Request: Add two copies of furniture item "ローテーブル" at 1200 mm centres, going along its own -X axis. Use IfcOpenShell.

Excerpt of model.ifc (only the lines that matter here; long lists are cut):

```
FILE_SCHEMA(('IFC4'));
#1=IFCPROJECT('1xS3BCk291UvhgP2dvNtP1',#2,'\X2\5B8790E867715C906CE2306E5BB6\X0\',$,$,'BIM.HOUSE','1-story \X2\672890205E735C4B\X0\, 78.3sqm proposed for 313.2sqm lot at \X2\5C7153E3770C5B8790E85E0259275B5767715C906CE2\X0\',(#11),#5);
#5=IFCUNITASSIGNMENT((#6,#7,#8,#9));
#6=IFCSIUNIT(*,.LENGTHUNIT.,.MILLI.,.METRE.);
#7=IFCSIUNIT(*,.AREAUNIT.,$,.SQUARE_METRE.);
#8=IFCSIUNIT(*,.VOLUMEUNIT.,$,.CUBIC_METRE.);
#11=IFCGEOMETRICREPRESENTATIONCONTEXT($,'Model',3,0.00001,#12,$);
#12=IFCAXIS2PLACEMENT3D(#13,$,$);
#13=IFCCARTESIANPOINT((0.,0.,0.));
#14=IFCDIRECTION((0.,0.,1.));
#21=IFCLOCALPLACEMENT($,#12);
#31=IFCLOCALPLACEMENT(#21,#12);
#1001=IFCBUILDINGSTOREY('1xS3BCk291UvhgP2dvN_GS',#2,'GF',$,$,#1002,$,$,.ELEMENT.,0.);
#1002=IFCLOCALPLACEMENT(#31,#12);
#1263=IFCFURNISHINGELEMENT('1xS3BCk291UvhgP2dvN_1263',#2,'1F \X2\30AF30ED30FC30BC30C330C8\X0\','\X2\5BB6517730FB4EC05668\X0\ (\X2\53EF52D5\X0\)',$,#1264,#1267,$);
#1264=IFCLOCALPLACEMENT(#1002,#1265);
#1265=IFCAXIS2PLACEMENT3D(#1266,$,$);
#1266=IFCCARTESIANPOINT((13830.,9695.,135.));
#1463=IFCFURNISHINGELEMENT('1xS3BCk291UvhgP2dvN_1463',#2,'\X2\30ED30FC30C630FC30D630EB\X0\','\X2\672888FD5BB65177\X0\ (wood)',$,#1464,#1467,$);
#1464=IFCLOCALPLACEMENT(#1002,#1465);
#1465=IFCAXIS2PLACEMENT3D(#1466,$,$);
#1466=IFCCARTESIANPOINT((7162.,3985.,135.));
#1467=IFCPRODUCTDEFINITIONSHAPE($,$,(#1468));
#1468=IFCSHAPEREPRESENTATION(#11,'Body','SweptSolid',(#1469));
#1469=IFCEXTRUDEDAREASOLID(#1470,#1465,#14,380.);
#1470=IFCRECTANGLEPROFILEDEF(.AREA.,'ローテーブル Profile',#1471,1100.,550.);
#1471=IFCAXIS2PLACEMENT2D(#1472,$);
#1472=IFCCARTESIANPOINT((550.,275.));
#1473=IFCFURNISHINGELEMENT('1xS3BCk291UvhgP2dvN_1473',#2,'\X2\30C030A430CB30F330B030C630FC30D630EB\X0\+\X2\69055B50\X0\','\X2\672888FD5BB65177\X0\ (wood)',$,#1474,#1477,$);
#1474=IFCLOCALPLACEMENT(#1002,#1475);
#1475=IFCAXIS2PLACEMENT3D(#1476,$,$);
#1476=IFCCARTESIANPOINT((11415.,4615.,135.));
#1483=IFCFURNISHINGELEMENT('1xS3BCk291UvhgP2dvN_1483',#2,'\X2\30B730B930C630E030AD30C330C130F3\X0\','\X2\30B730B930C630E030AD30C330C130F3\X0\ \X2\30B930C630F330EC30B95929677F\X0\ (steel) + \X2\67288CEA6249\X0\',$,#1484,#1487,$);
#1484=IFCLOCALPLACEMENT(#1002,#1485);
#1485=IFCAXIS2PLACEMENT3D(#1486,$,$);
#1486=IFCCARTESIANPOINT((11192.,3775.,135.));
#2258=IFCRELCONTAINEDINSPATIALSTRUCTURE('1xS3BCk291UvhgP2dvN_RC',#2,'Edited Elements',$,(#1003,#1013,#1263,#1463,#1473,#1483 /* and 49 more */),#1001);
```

```python
import ifcopenshell
import ifcopenshell.api.geometry
import ifcopenshell.api.root
import ifcopenshell.util.element
import ifcopenshell.util.placement

model = ifcopenshell.open("model.ifc")


def reuse_history(source, copy):
    """copy_class also copies each property set's owner history, people and application; keep the originals."""
    for rel in copy.IsDefinedBy:
        if rel.is_a("IfcRelDefinesByProperties") and (history := rel.RelatingPropertyDefinition.OwnerHistory):
            rel.RelatingPropertyDefinition.OwnerHistory = source.OwnerHistory
            ifcopenshell.util.element.remove_deep2(model, history)


source = model.by_guid("1xS3BCk291UvhgP2dvN_1463")
base = ifcopenshell.util.placement.get_local_placement(source.ObjectPlacement)
step = -base[:3, 0] * 1200.0

for i in range(1, 3):
    copy = ifcopenshell.api.root.copy_class(model, product=source)
    copy.Representation = ifcopenshell.util.element.copy_deep(
        model, source.Representation, exclude=["IfcGeometricRepresentationContext", "IfcRepresentationMap"]
    )
    reuse_history(source, copy)
    matrix = base.copy()
    matrix[:3, 3] += i * step
    print("added at", matrix[:3, 3].round(3) + 0.0)
    ifcopenshell.api.geometry.edit_object_placement(model, product=copy, matrix=matrix, is_si=False)

model.write("model_edited.ifc")
```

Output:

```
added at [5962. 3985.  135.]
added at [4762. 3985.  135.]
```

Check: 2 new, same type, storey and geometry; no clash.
